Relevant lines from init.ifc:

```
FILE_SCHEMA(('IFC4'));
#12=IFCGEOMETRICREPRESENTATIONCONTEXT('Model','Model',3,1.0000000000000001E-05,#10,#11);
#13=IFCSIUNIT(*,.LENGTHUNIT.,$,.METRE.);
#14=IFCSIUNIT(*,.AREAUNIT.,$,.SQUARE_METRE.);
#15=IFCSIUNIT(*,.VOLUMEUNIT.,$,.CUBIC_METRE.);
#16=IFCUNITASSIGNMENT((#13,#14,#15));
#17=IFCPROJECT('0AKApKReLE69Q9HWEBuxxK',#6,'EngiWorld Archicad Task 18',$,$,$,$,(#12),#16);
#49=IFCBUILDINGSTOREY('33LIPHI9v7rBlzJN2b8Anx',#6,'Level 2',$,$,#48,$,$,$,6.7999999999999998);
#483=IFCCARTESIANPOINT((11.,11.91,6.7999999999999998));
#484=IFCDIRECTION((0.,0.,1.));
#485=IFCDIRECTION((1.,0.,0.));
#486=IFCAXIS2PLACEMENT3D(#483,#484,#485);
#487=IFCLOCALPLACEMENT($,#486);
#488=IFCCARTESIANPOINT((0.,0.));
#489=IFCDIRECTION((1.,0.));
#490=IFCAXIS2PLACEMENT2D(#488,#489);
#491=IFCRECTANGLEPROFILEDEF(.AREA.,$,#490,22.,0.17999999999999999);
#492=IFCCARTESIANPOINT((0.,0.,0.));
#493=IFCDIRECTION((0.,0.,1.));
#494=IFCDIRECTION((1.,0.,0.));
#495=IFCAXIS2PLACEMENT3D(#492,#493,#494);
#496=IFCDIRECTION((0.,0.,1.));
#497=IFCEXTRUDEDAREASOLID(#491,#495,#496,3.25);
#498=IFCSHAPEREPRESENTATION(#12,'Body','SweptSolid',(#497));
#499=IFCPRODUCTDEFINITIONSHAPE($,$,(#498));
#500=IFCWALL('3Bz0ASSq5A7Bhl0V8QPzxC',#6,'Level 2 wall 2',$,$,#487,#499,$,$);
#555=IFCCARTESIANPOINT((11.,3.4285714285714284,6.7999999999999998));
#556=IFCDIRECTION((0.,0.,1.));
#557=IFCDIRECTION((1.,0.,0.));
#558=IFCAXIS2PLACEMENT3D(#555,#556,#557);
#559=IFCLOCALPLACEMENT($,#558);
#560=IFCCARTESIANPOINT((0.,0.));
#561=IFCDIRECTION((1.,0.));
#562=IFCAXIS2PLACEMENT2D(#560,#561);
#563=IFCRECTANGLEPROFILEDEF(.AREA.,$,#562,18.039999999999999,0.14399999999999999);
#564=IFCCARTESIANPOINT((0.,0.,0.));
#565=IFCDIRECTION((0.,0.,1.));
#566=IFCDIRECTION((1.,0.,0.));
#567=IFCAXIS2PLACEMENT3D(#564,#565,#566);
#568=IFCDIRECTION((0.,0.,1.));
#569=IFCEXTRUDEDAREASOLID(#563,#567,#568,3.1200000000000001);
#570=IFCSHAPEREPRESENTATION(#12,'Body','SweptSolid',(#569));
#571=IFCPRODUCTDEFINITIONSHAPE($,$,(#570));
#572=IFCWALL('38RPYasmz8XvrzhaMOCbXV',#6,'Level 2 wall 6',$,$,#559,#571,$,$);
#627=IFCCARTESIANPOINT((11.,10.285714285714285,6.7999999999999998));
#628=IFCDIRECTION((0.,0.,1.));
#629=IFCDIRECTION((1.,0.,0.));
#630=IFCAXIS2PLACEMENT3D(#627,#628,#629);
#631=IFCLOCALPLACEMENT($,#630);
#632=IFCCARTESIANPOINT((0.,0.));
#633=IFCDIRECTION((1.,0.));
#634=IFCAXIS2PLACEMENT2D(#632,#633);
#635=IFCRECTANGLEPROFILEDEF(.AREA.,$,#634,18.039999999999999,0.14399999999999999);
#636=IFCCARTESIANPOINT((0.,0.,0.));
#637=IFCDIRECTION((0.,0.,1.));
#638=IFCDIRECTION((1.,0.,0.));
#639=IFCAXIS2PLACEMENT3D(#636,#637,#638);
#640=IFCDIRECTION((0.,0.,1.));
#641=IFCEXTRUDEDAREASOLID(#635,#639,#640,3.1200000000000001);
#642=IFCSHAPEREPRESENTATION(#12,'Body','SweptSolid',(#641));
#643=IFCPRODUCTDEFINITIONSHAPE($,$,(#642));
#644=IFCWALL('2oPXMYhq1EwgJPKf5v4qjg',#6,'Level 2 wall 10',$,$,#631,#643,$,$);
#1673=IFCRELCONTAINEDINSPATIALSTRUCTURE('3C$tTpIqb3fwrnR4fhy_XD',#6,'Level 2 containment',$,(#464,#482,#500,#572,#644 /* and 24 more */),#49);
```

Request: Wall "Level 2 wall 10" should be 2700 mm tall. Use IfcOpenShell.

```python
import ifcopenshell
import ifcopenshell.geom
import ifcopenshell.util.shape
import ifcopenshell.util.unit

model = ifcopenshell.open("init.ifc")
unit_scale = ifcopenshell.util.unit.calculate_unit_scale(model)
settings = ifcopenshell.geom.settings()


def volume(element):
    """Net volume in cubic metres, openings subtracted."""
    shape = ifcopenshell.geom.create_shape(settings, element)
    return ifcopenshell.util.shape.get_volume(shape.geometry)


wall = model.by_guid("2oPXMYhq1EwgJPKf5v4qjg")
before = volume(wall)

body = next(r for r in wall.Representation.Representations if r.RepresentationIdentifier == "Body")
solid = body.Items[0]
old_height = solid.Depth
solid.Depth = 2.7 / unit_scale
after = volume(wall)

print(f"height {old_height:g} -> {solid.Depth:g}, volume {before:.3f} -> {after:.3f} m3")

model.write("init_edited.ifc")
```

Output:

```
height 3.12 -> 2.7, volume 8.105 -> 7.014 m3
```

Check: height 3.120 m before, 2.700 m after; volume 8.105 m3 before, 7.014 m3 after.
